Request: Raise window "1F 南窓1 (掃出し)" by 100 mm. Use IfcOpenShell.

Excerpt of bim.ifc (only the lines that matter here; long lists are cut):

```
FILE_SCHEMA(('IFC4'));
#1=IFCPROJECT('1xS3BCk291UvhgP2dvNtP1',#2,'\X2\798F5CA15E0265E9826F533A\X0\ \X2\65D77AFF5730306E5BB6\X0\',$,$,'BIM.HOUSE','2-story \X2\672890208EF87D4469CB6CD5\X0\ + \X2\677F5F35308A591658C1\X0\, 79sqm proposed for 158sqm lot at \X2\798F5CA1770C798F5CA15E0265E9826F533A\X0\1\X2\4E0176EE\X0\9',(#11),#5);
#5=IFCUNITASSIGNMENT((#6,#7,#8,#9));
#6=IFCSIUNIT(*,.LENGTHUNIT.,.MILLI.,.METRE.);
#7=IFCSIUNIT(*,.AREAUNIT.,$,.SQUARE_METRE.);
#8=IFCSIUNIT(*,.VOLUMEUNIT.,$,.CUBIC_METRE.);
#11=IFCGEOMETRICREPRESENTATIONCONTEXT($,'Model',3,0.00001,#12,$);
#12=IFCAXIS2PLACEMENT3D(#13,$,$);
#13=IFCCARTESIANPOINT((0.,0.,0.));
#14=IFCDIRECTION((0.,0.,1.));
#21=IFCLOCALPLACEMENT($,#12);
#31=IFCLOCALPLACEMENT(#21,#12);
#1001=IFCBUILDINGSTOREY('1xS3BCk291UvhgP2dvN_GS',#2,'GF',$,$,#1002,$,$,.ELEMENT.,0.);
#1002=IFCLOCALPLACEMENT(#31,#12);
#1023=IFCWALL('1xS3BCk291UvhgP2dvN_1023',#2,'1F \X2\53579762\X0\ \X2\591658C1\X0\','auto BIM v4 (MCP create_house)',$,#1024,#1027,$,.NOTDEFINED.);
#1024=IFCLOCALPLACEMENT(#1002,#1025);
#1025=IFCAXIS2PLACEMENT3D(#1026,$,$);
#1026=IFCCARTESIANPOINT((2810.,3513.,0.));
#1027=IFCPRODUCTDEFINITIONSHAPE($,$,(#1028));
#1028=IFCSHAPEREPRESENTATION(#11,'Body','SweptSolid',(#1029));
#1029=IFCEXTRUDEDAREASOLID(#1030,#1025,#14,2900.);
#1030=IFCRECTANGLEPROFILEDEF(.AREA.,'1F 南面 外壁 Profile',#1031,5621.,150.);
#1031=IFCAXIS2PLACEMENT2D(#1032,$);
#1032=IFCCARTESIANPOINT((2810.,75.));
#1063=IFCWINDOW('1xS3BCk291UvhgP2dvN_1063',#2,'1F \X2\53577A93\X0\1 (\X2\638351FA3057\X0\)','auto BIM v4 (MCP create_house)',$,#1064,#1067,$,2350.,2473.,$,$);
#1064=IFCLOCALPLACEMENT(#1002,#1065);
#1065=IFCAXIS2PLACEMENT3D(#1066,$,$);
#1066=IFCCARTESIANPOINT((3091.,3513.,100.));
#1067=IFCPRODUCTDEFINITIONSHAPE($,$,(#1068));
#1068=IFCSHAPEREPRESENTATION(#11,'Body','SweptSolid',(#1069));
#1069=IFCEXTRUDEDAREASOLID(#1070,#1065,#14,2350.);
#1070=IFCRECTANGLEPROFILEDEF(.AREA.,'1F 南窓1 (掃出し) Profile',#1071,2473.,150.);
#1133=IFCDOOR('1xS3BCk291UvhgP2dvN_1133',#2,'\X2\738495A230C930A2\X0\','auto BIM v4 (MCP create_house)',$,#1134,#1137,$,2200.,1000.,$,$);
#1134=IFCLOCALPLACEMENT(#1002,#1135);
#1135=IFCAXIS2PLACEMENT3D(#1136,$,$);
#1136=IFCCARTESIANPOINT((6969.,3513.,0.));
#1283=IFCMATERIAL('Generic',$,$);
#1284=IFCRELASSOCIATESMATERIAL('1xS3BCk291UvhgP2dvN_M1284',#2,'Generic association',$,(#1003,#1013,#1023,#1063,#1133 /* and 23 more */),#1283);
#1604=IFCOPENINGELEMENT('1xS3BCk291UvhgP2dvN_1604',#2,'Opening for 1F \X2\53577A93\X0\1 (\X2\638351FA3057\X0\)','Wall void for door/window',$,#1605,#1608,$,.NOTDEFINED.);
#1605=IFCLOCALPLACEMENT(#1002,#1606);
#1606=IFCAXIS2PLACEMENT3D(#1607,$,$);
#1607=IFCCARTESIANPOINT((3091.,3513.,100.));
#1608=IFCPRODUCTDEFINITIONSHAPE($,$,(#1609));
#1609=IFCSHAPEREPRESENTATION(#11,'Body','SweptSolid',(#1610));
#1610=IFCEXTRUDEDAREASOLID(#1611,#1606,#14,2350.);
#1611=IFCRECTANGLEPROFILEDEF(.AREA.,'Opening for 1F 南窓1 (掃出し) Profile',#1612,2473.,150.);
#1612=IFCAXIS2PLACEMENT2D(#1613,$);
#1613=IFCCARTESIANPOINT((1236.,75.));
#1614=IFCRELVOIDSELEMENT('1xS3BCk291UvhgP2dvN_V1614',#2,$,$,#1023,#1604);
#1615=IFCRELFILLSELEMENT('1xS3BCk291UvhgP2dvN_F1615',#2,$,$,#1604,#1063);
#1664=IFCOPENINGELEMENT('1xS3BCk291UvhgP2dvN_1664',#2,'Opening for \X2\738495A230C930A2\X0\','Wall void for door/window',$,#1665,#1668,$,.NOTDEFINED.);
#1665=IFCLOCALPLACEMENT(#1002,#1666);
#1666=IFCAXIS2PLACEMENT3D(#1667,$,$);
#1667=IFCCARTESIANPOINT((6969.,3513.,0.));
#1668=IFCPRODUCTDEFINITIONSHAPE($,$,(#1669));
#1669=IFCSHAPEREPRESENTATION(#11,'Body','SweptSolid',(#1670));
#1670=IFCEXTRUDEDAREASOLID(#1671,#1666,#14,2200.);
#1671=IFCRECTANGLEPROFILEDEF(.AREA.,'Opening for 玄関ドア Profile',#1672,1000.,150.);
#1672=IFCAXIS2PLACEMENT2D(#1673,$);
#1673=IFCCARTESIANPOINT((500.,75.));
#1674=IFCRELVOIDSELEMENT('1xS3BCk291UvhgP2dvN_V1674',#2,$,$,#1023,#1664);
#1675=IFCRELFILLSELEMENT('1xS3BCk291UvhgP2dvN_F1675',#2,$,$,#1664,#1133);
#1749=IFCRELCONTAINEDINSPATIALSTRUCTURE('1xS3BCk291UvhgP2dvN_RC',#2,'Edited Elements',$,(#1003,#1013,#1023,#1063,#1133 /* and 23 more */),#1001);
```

```python
import numpy as np
import ifcopenshell
import ifcopenshell.api.geometry
import ifcopenshell.util.placement
import ifcopenshell.util.unit

model = ifcopenshell.open("bim.ifc")
unit_scale = ifcopenshell.util.unit.calculate_unit_scale(model)

window = model.by_guid("1xS3BCk291UvhgP2dvN_1063")
opening = window.FillsVoids[0].RelatingOpeningElement
dz = 100.0

shift = np.array([0.0, 0.0, dz])
# The window is not placed relative to its opening, so move both.
for product in (opening, window):
    matrix = ifcopenshell.util.placement.get_local_placement(product.ObjectPlacement)
    matrix[:3, 3] += shift
    ifcopenshell.api.geometry.edit_object_placement(model, product=product, matrix=matrix, is_si=False)

print(f"moved by {dz * unit_scale:+.3f} m")

model.write("bim_rev.ifc")
```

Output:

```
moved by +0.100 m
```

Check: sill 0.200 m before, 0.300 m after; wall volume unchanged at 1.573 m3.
